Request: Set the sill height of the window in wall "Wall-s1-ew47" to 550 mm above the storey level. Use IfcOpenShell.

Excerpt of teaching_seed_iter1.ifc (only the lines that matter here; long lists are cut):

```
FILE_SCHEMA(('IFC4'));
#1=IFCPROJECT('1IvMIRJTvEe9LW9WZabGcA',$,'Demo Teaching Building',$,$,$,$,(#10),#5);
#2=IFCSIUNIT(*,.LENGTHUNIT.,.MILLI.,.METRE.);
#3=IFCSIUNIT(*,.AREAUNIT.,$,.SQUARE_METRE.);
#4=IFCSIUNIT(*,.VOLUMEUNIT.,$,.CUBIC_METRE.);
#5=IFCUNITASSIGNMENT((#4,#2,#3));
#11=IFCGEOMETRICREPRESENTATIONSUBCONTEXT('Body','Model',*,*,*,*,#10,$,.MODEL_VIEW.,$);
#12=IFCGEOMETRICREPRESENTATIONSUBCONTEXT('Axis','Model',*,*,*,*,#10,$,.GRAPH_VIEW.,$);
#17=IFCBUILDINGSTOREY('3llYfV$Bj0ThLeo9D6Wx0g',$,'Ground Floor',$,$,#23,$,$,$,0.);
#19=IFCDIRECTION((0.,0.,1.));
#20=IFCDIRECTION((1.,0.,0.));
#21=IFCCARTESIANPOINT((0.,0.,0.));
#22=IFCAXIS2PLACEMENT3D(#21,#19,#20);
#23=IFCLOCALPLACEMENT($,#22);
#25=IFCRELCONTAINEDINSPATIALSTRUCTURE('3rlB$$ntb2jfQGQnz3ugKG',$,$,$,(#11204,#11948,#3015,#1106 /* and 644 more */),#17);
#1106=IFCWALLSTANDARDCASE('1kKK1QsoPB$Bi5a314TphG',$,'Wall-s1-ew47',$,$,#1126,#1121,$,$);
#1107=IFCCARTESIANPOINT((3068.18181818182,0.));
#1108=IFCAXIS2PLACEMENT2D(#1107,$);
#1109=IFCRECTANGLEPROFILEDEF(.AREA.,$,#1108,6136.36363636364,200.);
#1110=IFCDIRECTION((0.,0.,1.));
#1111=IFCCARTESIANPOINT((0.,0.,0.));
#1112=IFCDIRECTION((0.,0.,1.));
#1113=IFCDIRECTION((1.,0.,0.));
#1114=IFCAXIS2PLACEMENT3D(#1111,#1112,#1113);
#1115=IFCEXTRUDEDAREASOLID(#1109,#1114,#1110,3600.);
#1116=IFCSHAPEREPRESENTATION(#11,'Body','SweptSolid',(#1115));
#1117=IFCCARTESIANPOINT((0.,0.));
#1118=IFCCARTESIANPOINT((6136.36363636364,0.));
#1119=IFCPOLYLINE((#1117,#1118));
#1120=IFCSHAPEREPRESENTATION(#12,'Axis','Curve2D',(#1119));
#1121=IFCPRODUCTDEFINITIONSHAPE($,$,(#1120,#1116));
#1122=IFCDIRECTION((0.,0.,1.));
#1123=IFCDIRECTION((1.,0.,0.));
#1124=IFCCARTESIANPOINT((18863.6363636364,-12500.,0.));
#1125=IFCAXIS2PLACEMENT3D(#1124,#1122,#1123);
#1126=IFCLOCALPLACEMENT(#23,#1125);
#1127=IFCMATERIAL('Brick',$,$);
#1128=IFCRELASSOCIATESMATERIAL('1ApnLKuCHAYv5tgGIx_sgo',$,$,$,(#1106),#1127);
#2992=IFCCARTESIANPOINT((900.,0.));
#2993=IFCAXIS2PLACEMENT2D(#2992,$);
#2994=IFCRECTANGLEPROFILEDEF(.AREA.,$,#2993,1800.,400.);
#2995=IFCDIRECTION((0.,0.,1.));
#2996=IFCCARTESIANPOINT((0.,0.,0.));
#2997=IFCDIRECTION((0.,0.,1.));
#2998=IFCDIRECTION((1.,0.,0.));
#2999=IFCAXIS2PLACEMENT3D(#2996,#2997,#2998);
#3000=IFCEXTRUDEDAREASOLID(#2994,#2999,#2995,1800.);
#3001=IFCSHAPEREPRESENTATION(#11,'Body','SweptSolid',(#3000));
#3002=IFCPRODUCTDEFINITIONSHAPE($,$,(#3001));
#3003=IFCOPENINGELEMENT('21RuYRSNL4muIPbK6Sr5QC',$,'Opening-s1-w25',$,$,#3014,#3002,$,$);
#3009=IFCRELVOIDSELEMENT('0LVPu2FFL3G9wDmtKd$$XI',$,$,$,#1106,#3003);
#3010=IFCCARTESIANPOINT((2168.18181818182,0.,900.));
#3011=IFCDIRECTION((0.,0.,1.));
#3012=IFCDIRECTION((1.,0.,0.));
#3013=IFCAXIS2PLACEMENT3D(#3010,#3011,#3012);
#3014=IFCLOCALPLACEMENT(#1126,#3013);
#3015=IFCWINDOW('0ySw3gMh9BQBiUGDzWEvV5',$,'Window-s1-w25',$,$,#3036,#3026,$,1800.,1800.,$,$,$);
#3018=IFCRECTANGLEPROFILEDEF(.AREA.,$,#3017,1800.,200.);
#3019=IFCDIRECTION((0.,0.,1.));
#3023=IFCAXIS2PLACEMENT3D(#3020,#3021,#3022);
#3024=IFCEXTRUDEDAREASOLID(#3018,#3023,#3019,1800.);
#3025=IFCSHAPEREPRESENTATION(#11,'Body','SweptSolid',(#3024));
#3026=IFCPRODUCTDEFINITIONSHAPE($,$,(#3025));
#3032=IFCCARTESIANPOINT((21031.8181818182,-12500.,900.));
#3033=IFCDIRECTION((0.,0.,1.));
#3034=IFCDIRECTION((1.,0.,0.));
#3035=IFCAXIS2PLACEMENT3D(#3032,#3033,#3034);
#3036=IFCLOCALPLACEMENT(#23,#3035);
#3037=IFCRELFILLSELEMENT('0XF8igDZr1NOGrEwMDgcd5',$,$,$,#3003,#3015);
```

```python
import numpy as np
import ifcopenshell
import ifcopenshell.api.geometry
import ifcopenshell.geom
import ifcopenshell.util.element
import ifcopenshell.util.placement
import ifcopenshell.util.shape
import ifcopenshell.util.unit

model = ifcopenshell.open("teaching_seed_iter1.ifc")
unit_scale = ifcopenshell.util.unit.calculate_unit_scale(model)

window = model.by_id(3015)
opening = window.FillsVoids[0].RelatingOpeningElement
storey = ifcopenshell.util.element.get_container(window, ifc_class="IfcBuildingStorey")
level = ifcopenshell.util.placement.get_local_placement(storey.ObjectPlacement)[2, 3]

# The opening's origin need not be at the sill, so measure its lowest point.
shape = ifcopenshell.geom.create_shape(ifcopenshell.geom.settings(), opening)
bottom = ifcopenshell.util.shape.get_shape_bottom_elevation(shape, shape.geometry) / unit_scale
dz = level + 0.55 / unit_scale - bottom

shift = np.array([0.0, 0.0, dz])
# The window is not placed relative to its opening, so move both.
for product in (opening, window):
    matrix = ifcopenshell.util.placement.get_local_placement(product.ObjectPlacement)
    matrix[:3, 3] += shift
    ifcopenshell.api.geometry.edit_object_placement(model, product=product, matrix=matrix, is_si=False)

print(f"moved by {dz * unit_scale:+.3f} m")

model.write("teaching_seed_iter1_rev.ifc")
```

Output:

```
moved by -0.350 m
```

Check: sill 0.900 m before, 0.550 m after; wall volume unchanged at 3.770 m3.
